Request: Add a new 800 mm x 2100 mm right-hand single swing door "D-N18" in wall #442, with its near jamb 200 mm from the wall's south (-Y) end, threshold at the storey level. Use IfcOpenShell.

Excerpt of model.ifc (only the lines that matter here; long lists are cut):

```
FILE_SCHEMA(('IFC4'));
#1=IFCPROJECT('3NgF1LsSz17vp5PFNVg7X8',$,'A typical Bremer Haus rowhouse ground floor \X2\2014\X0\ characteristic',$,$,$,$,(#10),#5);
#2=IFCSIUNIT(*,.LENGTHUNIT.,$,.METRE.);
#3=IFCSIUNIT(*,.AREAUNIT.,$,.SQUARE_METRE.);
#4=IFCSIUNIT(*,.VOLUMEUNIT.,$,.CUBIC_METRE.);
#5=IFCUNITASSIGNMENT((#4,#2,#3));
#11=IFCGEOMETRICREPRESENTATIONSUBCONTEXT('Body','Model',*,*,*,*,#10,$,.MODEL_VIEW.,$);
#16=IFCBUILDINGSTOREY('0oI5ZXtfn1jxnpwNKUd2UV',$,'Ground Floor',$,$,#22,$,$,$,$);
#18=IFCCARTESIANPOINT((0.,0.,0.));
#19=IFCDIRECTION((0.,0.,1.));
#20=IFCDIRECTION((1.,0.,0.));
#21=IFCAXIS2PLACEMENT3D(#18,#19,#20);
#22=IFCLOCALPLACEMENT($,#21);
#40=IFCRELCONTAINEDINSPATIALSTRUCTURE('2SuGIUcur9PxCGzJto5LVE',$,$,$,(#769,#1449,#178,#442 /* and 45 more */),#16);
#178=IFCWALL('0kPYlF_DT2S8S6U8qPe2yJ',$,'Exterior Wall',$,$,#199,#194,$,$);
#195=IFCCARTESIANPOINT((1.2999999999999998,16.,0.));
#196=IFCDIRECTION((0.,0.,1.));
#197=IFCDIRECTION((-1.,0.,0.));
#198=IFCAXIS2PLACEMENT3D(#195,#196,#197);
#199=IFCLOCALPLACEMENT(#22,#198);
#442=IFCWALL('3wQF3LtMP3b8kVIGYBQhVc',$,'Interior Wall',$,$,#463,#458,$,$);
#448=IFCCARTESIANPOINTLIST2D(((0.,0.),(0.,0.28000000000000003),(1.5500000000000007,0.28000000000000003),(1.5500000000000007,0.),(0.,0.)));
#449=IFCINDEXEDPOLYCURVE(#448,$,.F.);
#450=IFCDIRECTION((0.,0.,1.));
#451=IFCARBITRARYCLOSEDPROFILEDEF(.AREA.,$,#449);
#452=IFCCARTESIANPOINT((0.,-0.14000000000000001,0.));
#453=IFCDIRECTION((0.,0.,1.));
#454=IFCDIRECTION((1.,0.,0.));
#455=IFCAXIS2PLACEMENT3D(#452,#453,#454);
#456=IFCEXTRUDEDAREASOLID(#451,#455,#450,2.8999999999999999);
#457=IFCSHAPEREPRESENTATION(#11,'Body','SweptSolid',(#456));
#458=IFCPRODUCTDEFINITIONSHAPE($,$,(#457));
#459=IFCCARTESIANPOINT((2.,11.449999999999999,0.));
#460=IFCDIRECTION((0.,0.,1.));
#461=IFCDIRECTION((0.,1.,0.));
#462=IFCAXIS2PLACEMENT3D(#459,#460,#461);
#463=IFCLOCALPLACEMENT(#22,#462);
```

```python
import numpy as np
import ifcopenshell
import ifcopenshell.api.feature
import ifcopenshell.api.geometry
import ifcopenshell.api.root
import ifcopenshell.api.spatial
import ifcopenshell.geom
import ifcopenshell.util.element
import ifcopenshell.util.placement
import ifcopenshell.util.representation
import ifcopenshell.util.shape
import ifcopenshell.util.unit

model = ifcopenshell.open("model.ifc")
unit_scale = ifcopenshell.util.unit.calculate_unit_scale(model)
settings = ifcopenshell.geom.settings()


def volume(element):
    """Net volume in cubic metres, openings subtracted."""
    shape = ifcopenshell.geom.create_shape(settings, element)
    return ifcopenshell.util.shape.get_volume(shape.geometry)


wall = model.by_id(442)
storey = ifcopenshell.util.element.get_container(wall, ifc_class="IfcBuildingStorey")
context = ifcopenshell.util.representation.get_context(model, "Model", "Body", "MODEL_VIEW")
before = volume(wall)

width, height, from_end, sill = 0.8, 2.1, 0.2, 0.0  # metres

# The wall runs along its own X axis, and the end named is its -X end.
wall_shape = ifcopenshell.geom.create_shape(settings, wall)
x, y, z = ifcopenshell.util.shape.get_vertices(wall_shape.geometry).T
start = x.min() + from_end
face, thickness = float(y.min()), float(y.max() - y.min())
wall_matrix = ifcopenshell.util.placement.get_local_placement(wall.ObjectPlacement)
level = ifcopenshell.util.placement.get_local_placement(storey.ObjectPlacement)[2, 3]


def in_wall(x, y):
    """Placement at x, y metres in the wall's axes, at sill height."""
    matrix = wall_matrix.copy()
    matrix[:, 3] = wall_matrix @ np.array([x / unit_scale, y / unit_scale, 0.0, 1.0])
    matrix[2, 3] = level + sill / unit_scale
    return matrix


# Opening: a box that overshoots both wall faces by 50 mm.
opening = ifcopenshell.api.root.create_entity(model, ifc_class="IfcOpeningElement", predefined_type="OPENING")
box = ifcopenshell.api.geometry.add_wall_representation(
    model, context=context, length=width, height=height, thickness=thickness + 0.1
)
ifcopenshell.api.geometry.assign_representation(model, product=opening, representation=box)
ifcopenshell.api.geometry.edit_object_placement(model, product=opening, matrix=in_wall(start, face - 0.05), is_si=False)
ifcopenshell.api.feature.add_feature(model, feature=opening, element=wall)

door = ifcopenshell.api.root.create_entity(model, ifc_class="IfcDoor", name="D-N18", predefined_type="DOOR")
door.OverallWidth, door.OverallHeight = width / unit_scale, height / unit_scale
door.OperationType = "SINGLE_SWING_RIGHT"
body = ifcopenshell.api.geometry.add_door_representation(
    model,
    context=context,
    overall_width=door.OverallWidth,
    overall_height=door.OverallHeight,
    operation_type="SINGLE_SWING_RIGHT",
    lining_properties={"LiningDepth": thickness / unit_scale, "ThresholdDepth": thickness / unit_scale},
)
ifcopenshell.api.geometry.assign_representation(model, product=door, representation=body)
ifcopenshell.api.spatial.assign_container(model, products=[door], relating_structure=storey)
ifcopenshell.api.feature.add_filling(model, opening=opening, element=door)

# The lining spans the wall, so the door starts at the wall face.
ifcopenshell.api.geometry.edit_object_placement(model, product=door, matrix=in_wall(start, face), is_si=False)

after = volume(wall)

print(f"wall volume {before:.3f} -> {after:.3f} m3")

model.write("model_v2.ifc")
```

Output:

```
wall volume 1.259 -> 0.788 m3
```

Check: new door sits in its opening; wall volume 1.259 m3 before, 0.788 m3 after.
